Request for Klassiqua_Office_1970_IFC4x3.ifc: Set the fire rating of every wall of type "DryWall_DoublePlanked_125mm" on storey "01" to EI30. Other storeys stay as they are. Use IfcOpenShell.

First a look at what the model holds.

```python
import ifcopenshell
import ifcopenshell.util.element

model = ifcopenshell.open("Klassiqua_Office_1970_IFC4x3.ifc")
print(model.schema)
storey = next(s for s in model.by_type("IfcBuildingStorey") if s.Name == "01")
walls = [e for e in ifcopenshell.util.element.get_decomposition(storey) if e.is_a("IfcWall")]
seen = {}
for e in walls:
    element_type = ifcopenshell.util.element.get_type(e)
    key = (element_type.Name if element_type != e and element_type else None, ifcopenshell.util.element.get_pset(e, "Pset_WallCommon", "FireRating"))
    seen[key] = seen.get(key, 0) + 1
for (name, value), count in sorted(seen.items(), key=str):
    print(count, "x", name, "|", value)
```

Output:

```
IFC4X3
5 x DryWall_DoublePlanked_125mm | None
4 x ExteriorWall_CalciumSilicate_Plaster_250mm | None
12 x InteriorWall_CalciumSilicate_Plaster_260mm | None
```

```python
import ifcopenshell
import ifcopenshell.api.pset
import ifcopenshell.util.element

model = ifcopenshell.open("Klassiqua_Office_1970_IFC4x3.ifc")

storey = next(s for s in model.by_type("IfcBuildingStorey") if s.Name == "01")
walls = [e for e in ifcopenshell.util.element.get_decomposition(storey) if e.is_a("IfcWall")]

count = 0
for e in walls:
    element_type = ifcopenshell.util.element.get_type(e)
    if element_type in (None, e) or element_type.Name != "DryWall_DoublePlanked_125mm":
        continue
    # add_pset returns the element's existing set when there is one.
    pset = ifcopenshell.api.pset.add_pset(model, product=e, name="Pset_WallCommon")
    ifcopenshell.api.pset.edit_pset(model, pset=pset, properties={"FireRating": "EI30"})
    count += 1

print(count, "walls updated")

model.write("Klassiqua_Office_1970_IFC4x3-out.ifc")
```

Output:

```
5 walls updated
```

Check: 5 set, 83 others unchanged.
